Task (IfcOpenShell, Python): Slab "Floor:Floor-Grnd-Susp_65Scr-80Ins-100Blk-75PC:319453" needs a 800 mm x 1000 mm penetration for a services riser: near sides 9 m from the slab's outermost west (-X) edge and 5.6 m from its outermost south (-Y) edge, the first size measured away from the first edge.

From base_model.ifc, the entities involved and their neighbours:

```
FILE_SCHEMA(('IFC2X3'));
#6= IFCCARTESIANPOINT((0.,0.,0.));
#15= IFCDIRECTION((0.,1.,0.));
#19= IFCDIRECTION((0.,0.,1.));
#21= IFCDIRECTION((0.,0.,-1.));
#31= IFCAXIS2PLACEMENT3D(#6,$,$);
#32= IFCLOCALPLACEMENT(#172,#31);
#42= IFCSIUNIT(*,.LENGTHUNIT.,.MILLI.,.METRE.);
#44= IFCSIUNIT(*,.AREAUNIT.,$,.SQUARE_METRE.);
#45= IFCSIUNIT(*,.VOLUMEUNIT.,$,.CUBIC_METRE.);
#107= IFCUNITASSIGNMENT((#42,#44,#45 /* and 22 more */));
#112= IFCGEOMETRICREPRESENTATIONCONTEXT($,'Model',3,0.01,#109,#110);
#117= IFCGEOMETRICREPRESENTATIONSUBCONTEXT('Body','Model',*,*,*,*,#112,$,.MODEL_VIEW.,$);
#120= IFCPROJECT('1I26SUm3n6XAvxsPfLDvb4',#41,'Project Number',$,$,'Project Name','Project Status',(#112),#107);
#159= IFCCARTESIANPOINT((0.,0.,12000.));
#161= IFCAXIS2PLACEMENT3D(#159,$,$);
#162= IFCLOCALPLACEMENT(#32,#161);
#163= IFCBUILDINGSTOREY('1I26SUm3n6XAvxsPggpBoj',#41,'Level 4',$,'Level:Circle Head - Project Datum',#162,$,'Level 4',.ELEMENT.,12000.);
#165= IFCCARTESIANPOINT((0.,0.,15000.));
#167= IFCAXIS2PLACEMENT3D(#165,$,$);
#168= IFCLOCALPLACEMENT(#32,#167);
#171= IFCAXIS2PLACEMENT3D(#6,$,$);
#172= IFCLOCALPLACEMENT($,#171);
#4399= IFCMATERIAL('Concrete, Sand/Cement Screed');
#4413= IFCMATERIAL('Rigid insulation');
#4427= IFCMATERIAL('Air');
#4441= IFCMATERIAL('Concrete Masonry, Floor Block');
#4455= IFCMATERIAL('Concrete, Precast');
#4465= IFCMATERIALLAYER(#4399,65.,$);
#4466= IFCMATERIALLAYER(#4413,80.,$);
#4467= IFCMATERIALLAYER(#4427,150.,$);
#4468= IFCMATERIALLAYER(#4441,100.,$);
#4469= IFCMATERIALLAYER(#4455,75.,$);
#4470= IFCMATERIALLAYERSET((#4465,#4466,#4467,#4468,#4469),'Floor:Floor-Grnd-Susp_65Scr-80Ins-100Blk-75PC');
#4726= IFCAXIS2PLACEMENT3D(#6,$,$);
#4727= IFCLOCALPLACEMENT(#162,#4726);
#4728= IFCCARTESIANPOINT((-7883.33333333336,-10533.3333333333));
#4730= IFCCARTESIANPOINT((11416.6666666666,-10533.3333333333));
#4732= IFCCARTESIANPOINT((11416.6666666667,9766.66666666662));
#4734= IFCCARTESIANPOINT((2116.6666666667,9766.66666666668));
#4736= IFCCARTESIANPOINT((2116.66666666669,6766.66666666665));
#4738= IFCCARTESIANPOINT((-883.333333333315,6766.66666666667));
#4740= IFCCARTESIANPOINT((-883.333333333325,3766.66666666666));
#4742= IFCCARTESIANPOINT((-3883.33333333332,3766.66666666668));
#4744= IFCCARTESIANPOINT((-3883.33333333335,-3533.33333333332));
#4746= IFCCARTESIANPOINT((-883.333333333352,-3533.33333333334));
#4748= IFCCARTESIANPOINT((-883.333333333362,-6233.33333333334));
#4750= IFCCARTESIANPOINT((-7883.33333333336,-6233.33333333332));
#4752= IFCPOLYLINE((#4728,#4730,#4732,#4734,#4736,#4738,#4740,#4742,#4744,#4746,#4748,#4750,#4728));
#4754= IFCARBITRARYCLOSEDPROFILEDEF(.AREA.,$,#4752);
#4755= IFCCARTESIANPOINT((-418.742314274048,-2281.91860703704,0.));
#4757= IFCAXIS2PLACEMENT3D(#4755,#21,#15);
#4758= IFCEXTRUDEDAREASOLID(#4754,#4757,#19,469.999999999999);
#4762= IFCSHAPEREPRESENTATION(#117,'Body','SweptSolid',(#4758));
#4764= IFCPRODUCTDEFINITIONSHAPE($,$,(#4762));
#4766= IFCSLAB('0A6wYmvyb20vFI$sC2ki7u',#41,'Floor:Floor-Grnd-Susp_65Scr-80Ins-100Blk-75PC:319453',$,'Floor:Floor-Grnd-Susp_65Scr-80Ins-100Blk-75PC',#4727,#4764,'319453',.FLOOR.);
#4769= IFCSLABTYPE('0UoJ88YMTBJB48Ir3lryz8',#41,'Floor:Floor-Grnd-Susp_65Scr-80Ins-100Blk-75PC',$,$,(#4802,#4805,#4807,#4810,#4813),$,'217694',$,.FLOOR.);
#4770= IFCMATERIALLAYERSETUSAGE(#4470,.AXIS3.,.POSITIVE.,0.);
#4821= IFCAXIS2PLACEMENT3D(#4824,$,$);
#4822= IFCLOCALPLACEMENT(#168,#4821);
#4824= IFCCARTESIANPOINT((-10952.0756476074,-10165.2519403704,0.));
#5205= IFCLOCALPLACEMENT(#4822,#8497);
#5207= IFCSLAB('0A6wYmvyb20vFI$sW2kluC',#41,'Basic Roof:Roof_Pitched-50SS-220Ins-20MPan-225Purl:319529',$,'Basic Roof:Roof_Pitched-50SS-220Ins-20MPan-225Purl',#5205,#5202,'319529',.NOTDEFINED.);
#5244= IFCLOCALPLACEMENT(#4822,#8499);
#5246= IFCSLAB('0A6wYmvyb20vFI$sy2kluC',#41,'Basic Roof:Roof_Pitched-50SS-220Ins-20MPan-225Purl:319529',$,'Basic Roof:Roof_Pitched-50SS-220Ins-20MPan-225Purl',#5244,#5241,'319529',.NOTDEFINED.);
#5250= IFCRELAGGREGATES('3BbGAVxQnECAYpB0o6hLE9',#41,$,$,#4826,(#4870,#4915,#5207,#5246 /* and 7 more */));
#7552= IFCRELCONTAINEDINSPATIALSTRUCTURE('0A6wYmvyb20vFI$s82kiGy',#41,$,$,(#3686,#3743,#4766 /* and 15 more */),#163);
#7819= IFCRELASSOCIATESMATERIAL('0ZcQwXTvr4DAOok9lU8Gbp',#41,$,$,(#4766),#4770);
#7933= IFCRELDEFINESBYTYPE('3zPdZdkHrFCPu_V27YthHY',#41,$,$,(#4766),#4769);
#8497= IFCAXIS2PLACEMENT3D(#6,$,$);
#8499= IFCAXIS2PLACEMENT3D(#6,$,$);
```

```python
import numpy as np
import ifcopenshell
import ifcopenshell.api.feature
import ifcopenshell.api.geometry
import ifcopenshell.api.root
import ifcopenshell.geom
import ifcopenshell.util.placement
import ifcopenshell.util.representation
import ifcopenshell.util.shape
import ifcopenshell.util.unit

model = ifcopenshell.open("base_model.ifc")
unit_scale = ifcopenshell.util.unit.calculate_unit_scale(model)
settings = ifcopenshell.geom.settings()


def volume(element):
    """Net volume in cubic metres, openings subtracted."""
    shape = ifcopenshell.geom.create_shape(settings, element)
    return ifcopenshell.util.shape.get_volume(shape.geometry)


slab = model.by_id(4766)
before = volume(slab)

# Extent in the slab's own axes, in metres. The edges named are its -X and -Y sides.
slab_shape = ifcopenshell.geom.create_shape(settings, slab)
vertices = ifcopenshell.util.shape.get_vertices(slab_shape.geometry)
x_min, y_min, bottom = vertices.min(axis=0)
top = vertices[:, 2].max()

opening = ifcopenshell.api.root.create_entity(model, ifc_class="IfcOpeningElement", name="Services riser opening")
context = ifcopenshell.util.representation.get_context(model, "Model", "Body", "MODEL_VIEW")
width, depth = 0.8, 1
outline = [(0.0, 0.0), (width, 0.0), (width, depth), (0.0, depth), (0.0, 0.0)]
# Overshoot both faces by 50 mm so the cut is clean.
shape = ifcopenshell.api.geometry.add_slab_representation(
    model, context=context, depth=top - bottom + 0.1, polyline=outline
)
ifcopenshell.api.geometry.assign_representation(model, product=opening, representation=shape)

matrix = ifcopenshell.util.placement.get_local_placement(slab.ObjectPlacement)
matrix[:, 3] = matrix @ np.append(np.array([x_min + 9, y_min + 5.6, bottom - 0.05]) / unit_scale, 1.0)
ifcopenshell.api.geometry.edit_object_placement(model, product=opening, matrix=matrix, is_si=False)
ifcopenshell.api.feature.add_feature(model, feature=opening, element=slab)

after = volume(slab)

print(f"slab volume {before:.3f} -> {after:.3f} m3")

model.write("base_model-out.ifc")
```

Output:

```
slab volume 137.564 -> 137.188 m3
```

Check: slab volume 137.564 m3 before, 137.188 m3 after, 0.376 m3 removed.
